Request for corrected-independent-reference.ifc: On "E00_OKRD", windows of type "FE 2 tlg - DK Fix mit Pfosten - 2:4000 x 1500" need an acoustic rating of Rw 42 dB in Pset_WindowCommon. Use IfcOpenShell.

First a look at what the model holds.

```python
import ifcopenshell
import ifcopenshell.util.element

model = ifcopenshell.open("corrected-independent-reference.ifc")
print(model.schema)
storey = next(s for s in model.by_type("IfcBuildingStorey") if s.Name == "E00_OKRD")
windows = [e for e in ifcopenshell.util.element.get_decomposition(storey) if e.is_a("IfcWindow")]
seen = {}
for e in windows:
    element_type = ifcopenshell.util.element.get_type(e)
    key = (element_type.Name if element_type != e and element_type else None, ifcopenshell.util.element.get_pset(e, "Pset_WindowCommon", "AcousticRating"))
    seen[key] = seen.get(key, 0) + 1
for (name, value), count in sorted(seen.items(), key=str):
    print(count, "x", name, "|", value)
```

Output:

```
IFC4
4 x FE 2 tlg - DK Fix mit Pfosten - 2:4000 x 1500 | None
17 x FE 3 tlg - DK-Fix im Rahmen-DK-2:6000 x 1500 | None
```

```python
import ifcopenshell
import ifcopenshell.api.pset
import ifcopenshell.util.element

model = ifcopenshell.open("corrected-independent-reference.ifc")

storey = next(s for s in model.by_type("IfcBuildingStorey") if s.Name == "E00_OKRD")
windows = [e for e in ifcopenshell.util.element.get_decomposition(storey) if e.is_a("IfcWindow")]

count = 0
for e in windows:
    element_type = ifcopenshell.util.element.get_type(e)
    if element_type in (None, e) or element_type.Name != "FE 2 tlg - DK Fix mit Pfosten - 2:4000 x 1500":
        continue
    # add_pset returns the element's existing set when there is one.
    pset = ifcopenshell.api.pset.add_pset(model, product=e, name="Pset_WindowCommon")
    ifcopenshell.api.pset.edit_pset(model, pset=pset, properties={"AcousticRating": "Rw 42 dB"})
    count += 1

print(count, "windows updated")

model.write("corrected-independent-reference_v2.ifc")
```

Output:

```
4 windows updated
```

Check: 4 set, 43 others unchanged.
